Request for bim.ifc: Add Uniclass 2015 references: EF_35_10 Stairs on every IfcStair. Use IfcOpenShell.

First a look at what the model holds.

```python
import ifcopenshell

model = ifcopenshell.open("bim.ifc")
print(model.schema)
print("classifications:", [c.Name for c in model.by_type("IfcClassification")])
for ifc_class in ("IfcDoor", "IfcRoof", "IfcStair", "IfcWall", "IfcWindow"):
    print(ifc_class, len(model.by_type(ifc_class)))
```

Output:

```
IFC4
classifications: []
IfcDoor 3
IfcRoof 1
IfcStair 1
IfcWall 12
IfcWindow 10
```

```python
import ifcopenshell
import ifcopenshell.api.classification

model = ifcopenshell.open("bim.ifc")

system = ifcopenshell.api.classification.add_classification(model, classification="Uniclass 2015")

codes = {
    "IfcStair": ("EF_35_10", "Stairs"),
}
for ifc_class, (code, name) in codes.items():
    products = model.by_type(ifc_class)
    ifcopenshell.api.classification.add_reference(
        model, products=products, classification=system, identification=code, name=name
    )
    print(code, len(products))

model.write("bim_updated.ifc")
```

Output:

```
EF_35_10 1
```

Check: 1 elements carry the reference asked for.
